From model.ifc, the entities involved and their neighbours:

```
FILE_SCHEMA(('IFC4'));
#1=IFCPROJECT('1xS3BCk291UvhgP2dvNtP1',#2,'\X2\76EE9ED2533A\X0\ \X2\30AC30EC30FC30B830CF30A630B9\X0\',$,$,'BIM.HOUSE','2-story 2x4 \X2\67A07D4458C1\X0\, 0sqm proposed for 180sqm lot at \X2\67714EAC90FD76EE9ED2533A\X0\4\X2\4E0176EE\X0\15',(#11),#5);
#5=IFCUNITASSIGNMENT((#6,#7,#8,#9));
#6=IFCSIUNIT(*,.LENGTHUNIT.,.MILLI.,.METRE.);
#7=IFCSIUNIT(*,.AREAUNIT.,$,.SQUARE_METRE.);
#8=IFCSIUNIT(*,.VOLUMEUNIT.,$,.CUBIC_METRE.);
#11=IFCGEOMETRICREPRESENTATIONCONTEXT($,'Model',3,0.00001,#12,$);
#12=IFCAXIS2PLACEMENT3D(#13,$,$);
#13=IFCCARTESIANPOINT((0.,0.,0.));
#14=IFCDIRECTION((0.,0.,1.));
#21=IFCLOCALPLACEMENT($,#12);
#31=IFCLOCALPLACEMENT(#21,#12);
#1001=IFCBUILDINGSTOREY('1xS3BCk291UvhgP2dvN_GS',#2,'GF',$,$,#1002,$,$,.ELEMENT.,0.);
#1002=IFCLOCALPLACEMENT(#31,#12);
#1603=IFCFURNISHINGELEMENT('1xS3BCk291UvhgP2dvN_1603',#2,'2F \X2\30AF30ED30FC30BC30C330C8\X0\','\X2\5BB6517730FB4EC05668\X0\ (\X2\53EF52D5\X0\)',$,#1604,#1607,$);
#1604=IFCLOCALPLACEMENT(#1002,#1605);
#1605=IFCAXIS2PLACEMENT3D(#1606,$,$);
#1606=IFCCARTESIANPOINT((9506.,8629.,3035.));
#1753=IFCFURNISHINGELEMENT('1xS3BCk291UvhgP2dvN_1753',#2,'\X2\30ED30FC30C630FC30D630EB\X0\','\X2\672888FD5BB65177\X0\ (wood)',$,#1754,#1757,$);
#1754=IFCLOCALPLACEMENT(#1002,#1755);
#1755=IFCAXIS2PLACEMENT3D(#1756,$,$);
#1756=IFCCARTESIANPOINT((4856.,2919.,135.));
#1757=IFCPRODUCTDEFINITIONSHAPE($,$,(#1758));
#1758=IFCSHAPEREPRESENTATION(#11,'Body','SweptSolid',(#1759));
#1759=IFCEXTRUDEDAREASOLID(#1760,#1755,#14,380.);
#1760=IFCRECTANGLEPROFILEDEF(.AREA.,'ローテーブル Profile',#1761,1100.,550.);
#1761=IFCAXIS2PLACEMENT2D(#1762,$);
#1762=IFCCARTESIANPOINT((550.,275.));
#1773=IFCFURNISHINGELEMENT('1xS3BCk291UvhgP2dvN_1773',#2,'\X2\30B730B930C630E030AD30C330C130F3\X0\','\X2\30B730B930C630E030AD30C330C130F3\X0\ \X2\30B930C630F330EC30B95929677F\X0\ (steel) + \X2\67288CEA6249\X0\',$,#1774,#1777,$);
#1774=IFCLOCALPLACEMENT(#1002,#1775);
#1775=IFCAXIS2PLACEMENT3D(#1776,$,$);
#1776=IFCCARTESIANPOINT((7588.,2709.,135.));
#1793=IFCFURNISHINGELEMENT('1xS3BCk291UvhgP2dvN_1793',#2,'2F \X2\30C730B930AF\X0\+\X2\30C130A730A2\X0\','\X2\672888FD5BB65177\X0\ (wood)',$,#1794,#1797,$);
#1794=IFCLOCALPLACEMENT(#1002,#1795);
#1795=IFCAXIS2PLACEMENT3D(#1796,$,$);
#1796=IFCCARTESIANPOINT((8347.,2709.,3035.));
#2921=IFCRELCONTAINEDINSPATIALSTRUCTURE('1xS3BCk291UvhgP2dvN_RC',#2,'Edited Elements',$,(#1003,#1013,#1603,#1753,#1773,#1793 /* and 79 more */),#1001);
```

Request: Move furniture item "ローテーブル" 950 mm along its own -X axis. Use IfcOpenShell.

```python
import ifcopenshell
import ifcopenshell.api.geometry
import ifcopenshell.util.placement

model = ifcopenshell.open("model.ifc")

item = model.by_guid("1xS3BCk291UvhgP2dvN_1753")
matrix = ifcopenshell.util.placement.get_local_placement(item.ObjectPlacement)
matrix[:3, 3] -= matrix[:3, 0] * 950.0
ifcopenshell.api.geometry.edit_object_placement(model, product=item, matrix=matrix, is_si=False)

print(ifcopenshell.util.placement.get_local_placement(item.ObjectPlacement).round(3) + 0.0)

model.write("model_rev.ifc")
```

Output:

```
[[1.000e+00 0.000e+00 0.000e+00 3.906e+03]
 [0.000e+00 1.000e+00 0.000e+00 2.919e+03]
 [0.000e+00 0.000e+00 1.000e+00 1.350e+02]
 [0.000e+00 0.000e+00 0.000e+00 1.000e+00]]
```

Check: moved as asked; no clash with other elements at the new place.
